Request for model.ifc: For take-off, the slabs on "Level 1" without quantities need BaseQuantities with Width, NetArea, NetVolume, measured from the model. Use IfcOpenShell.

First a look at what the model holds.

```python
import ifcopenshell
import ifcopenshell.util.element
import ifcopenshell.util.unit

model = ifcopenshell.open("model.ifc")
print(model.schema)
for unit_type in ("LENGTHUNIT", "AREAUNIT", "VOLUMEUNIT"):
    print(unit_type, ifcopenshell.util.unit.calculate_unit_scale(model, unit_type))
storey = next(s for s in model.by_type("IfcBuildingStorey") if s.Name == "Level 1")
slabs = [e for e in ifcopenshell.util.element.get_decomposition(storey) if e.is_a("IfcSlab")]
for e in sorted(slabs, key=lambda e: e.id()):
    print(e.id(), e.is_a(), e.Name, list(ifcopenshell.util.element.get_psets(e, qtos_only=True)), sep=" | ")
```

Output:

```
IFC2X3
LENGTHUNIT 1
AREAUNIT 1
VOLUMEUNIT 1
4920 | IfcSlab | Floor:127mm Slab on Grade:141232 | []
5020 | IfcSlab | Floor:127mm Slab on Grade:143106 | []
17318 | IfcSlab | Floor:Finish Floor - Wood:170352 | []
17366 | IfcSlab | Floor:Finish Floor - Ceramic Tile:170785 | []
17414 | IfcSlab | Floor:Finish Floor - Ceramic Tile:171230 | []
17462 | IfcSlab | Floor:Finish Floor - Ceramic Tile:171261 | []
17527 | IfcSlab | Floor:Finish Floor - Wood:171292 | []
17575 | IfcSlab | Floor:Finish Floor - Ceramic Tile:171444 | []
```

```python
import ifcopenshell
import ifcopenshell.api.pset
import ifcopenshell.geom
import ifcopenshell.util.element
import ifcopenshell.util.shape
import ifcopenshell.util.unit

model = ifcopenshell.open("model.ifc")
unit_scale = ifcopenshell.util.unit.calculate_unit_scale(model)
area_scale = ifcopenshell.util.unit.calculate_unit_scale(model, "AREAUNIT")
volume_scale = ifcopenshell.util.unit.calculate_unit_scale(model, "VOLUMEUNIT")
settings = ifcopenshell.geom.settings()

storey = next(s for s in model.by_type("IfcBuildingStorey") if s.Name == "Level 1")
slabs = [e for e in ifcopenshell.util.element.get_decomposition(storey) if e.is_a("IfcSlab")]

for e in sorted(slabs, key=lambda e: e.id()):
    if ifcopenshell.util.element.get_psets(e, qtos_only=True, should_inherit=False):
        continue
    # Geometry comes back in metres, in the element's own axes.
    shape = ifcopenshell.geom.create_shape(settings, e)
    values = {
        "Width": ifcopenshell.util.shape.get_z(shape.geometry) / unit_scale,
        "NetArea": ifcopenshell.util.shape.get_footprint_area(shape.geometry) / area_scale,
        "NetVolume": ifcopenshell.util.shape.get_volume(shape.geometry) / volume_scale,
    }
    qto = ifcopenshell.api.pset.add_qto(model, product=e, name="BaseQuantities")
    ifcopenshell.api.pset.edit_qto(model, qto=qto, properties=values)
    print(e.id(), {k: round(v, 3) for k, v in values.items()})

model.write("model_rev.ifc")
```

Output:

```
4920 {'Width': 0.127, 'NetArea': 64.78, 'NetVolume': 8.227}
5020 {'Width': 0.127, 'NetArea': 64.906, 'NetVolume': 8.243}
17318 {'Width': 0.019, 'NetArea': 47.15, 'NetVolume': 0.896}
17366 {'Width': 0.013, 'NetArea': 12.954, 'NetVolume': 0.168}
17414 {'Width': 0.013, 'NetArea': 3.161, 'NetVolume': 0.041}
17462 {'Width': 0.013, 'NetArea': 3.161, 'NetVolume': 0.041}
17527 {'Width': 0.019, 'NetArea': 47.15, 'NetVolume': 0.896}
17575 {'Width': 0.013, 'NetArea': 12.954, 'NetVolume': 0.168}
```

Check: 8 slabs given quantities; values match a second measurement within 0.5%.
